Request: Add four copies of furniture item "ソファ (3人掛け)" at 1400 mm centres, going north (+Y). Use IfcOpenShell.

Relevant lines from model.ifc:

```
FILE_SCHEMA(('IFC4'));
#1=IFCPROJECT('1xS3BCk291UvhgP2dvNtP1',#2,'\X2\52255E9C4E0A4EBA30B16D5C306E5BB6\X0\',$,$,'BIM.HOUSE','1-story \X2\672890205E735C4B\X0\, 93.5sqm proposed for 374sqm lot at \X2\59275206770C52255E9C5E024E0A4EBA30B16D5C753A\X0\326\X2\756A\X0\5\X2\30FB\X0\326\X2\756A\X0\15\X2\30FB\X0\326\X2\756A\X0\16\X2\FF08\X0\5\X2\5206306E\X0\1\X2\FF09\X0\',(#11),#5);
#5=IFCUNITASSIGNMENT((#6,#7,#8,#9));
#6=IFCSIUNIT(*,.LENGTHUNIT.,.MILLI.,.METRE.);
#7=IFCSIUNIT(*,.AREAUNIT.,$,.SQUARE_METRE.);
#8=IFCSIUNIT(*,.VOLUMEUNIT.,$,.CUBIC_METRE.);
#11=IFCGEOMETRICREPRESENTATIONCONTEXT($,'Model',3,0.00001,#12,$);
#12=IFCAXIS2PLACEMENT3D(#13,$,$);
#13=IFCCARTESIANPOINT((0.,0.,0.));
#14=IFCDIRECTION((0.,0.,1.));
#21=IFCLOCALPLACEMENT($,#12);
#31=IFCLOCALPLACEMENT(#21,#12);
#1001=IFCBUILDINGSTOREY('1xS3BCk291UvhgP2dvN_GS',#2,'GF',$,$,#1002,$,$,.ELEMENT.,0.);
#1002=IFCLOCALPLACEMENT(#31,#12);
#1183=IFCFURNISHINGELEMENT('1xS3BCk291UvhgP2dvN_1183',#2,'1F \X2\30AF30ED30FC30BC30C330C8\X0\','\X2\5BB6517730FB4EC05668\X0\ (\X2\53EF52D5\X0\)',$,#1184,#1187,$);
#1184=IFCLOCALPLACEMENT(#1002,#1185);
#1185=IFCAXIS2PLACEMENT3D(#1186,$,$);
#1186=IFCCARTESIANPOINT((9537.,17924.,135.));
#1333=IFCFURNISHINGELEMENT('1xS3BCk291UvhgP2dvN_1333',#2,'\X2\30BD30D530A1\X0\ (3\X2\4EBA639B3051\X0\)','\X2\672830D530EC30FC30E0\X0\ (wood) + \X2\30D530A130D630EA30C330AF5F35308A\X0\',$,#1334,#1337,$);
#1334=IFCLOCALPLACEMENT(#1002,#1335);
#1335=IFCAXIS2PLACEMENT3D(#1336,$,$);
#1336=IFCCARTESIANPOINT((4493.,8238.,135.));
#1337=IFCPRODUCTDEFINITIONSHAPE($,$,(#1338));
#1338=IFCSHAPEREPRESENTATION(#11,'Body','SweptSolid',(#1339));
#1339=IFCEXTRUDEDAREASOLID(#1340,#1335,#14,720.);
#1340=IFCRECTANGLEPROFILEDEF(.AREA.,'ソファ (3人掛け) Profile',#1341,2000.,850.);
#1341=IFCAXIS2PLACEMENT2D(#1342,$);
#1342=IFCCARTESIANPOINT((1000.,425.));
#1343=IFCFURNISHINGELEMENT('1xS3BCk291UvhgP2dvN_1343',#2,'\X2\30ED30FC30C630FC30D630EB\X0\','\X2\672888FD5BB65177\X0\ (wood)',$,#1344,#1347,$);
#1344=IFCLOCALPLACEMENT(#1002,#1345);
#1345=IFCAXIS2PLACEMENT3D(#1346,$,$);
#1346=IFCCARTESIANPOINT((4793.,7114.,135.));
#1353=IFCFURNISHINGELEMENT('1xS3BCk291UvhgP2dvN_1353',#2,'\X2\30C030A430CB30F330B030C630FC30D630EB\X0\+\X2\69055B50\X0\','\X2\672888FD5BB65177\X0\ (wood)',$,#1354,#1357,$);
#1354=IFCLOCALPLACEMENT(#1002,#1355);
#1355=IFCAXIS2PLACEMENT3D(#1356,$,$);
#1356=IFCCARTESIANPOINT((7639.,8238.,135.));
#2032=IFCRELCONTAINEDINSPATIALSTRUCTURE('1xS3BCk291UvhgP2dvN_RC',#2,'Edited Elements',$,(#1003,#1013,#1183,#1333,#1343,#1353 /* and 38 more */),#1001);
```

```python
import numpy as np
import ifcopenshell
import ifcopenshell.api.geometry
import ifcopenshell.api.root
import ifcopenshell.util.element
import ifcopenshell.util.placement
import ifcopenshell.util.unit

model = ifcopenshell.open("model.ifc")
unit_scale = ifcopenshell.util.unit.calculate_unit_scale(model)


def reuse_history(source, copy):
    """copy_class also copies each property set's owner history, people and application; keep the originals."""
    for rel in copy.IsDefinedBy:
        if rel.is_a("IfcRelDefinesByProperties") and (history := rel.RelatingPropertyDefinition.OwnerHistory):
            rel.RelatingPropertyDefinition.OwnerHistory = source.OwnerHistory
            ifcopenshell.util.element.remove_deep2(model, history)


source = model.by_guid("1xS3BCk291UvhgP2dvN_1333")
base = ifcopenshell.util.placement.get_local_placement(source.ObjectPlacement)
step = np.array([0.0, 1.0, 0.0]) * 1.4 / unit_scale

for i in range(1, 5):
    copy = ifcopenshell.api.root.copy_class(model, product=source)
    copy.Representation = ifcopenshell.util.element.copy_deep(
        model, source.Representation, exclude=["IfcGeometricRepresentationContext", "IfcRepresentationMap"]
    )
    reuse_history(source, copy)
    matrix = base.copy()
    matrix[:3, 3] += i * step
    print("added at", matrix[:3, 3].round(3) + 0.0)
    ifcopenshell.api.geometry.edit_object_placement(model, product=copy, matrix=matrix, is_si=False)

model.write("model_rev.ifc")
```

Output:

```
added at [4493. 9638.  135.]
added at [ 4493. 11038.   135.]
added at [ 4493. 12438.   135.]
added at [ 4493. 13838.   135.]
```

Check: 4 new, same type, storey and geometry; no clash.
